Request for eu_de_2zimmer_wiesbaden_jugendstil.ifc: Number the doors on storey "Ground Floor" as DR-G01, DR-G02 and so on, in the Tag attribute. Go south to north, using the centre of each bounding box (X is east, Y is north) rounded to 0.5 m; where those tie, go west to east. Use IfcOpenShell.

First a look at what the model holds.

```python
import ifcopenshell
import ifcopenshell.util.element
import ifcopenshell.util.placement

model = ifcopenshell.open("eu_de_2zimmer_wiesbaden_jugendstil.ifc")
print(model.schema)
storey = next(s for s in model.by_type("IfcBuildingStorey") if s.Name == "Ground Floor")
doors = [e for e in ifcopenshell.util.element.get_decomposition(storey) if e.is_a("IfcDoor")]
for e in sorted(doors, key=lambda e: e.id()):
    origin = ifcopenshell.util.placement.get_local_placement(e.ObjectPlacement)[:3, 3]
    print(e.id(), e.Tag, e.Name, origin.round(2) + 0.0, sep=" | ")
```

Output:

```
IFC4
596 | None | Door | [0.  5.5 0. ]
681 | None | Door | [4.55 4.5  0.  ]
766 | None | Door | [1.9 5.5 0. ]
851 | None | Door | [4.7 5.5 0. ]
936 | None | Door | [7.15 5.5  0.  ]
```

```python
import ifcopenshell
import ifcopenshell.geom
import ifcopenshell.util.element
import ifcopenshell.util.shape

model = ifcopenshell.open("eu_de_2zimmer_wiesbaden_jugendstil.ifc")
settings = ifcopenshell.geom.settings()
settings.set("use-world-coords", True)


def centre(element):
    shape = ifcopenshell.geom.create_shape(settings, element)
    return ifcopenshell.util.shape.get_bbox_centroid(shape.geometry)


storey = next(s for s in model.by_type("IfcBuildingStorey") if s.Name == "Ground Floor")
doors = [e for e in ifcopenshell.util.element.get_decomposition(storey) if e.is_a("IfcDoor")]

# Insertion points can sit at a corner or the storey origin, so sort by the geometry (in metres).
centres = {e: centre(e) for e in doors}
doors.sort(key=lambda e: (round(centres[e][1] / 0.5), centres[e][0]))

for i, e in enumerate(doors, start=1):
    number = f"DR-G{i:02d}"
    e.Tag = number
    print(e.id(), number)

model.write("eu_de_2zimmer_wiesbaden_jugendstil_rev.ifc")
```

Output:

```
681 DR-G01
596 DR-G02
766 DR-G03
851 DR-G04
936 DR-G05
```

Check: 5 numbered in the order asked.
